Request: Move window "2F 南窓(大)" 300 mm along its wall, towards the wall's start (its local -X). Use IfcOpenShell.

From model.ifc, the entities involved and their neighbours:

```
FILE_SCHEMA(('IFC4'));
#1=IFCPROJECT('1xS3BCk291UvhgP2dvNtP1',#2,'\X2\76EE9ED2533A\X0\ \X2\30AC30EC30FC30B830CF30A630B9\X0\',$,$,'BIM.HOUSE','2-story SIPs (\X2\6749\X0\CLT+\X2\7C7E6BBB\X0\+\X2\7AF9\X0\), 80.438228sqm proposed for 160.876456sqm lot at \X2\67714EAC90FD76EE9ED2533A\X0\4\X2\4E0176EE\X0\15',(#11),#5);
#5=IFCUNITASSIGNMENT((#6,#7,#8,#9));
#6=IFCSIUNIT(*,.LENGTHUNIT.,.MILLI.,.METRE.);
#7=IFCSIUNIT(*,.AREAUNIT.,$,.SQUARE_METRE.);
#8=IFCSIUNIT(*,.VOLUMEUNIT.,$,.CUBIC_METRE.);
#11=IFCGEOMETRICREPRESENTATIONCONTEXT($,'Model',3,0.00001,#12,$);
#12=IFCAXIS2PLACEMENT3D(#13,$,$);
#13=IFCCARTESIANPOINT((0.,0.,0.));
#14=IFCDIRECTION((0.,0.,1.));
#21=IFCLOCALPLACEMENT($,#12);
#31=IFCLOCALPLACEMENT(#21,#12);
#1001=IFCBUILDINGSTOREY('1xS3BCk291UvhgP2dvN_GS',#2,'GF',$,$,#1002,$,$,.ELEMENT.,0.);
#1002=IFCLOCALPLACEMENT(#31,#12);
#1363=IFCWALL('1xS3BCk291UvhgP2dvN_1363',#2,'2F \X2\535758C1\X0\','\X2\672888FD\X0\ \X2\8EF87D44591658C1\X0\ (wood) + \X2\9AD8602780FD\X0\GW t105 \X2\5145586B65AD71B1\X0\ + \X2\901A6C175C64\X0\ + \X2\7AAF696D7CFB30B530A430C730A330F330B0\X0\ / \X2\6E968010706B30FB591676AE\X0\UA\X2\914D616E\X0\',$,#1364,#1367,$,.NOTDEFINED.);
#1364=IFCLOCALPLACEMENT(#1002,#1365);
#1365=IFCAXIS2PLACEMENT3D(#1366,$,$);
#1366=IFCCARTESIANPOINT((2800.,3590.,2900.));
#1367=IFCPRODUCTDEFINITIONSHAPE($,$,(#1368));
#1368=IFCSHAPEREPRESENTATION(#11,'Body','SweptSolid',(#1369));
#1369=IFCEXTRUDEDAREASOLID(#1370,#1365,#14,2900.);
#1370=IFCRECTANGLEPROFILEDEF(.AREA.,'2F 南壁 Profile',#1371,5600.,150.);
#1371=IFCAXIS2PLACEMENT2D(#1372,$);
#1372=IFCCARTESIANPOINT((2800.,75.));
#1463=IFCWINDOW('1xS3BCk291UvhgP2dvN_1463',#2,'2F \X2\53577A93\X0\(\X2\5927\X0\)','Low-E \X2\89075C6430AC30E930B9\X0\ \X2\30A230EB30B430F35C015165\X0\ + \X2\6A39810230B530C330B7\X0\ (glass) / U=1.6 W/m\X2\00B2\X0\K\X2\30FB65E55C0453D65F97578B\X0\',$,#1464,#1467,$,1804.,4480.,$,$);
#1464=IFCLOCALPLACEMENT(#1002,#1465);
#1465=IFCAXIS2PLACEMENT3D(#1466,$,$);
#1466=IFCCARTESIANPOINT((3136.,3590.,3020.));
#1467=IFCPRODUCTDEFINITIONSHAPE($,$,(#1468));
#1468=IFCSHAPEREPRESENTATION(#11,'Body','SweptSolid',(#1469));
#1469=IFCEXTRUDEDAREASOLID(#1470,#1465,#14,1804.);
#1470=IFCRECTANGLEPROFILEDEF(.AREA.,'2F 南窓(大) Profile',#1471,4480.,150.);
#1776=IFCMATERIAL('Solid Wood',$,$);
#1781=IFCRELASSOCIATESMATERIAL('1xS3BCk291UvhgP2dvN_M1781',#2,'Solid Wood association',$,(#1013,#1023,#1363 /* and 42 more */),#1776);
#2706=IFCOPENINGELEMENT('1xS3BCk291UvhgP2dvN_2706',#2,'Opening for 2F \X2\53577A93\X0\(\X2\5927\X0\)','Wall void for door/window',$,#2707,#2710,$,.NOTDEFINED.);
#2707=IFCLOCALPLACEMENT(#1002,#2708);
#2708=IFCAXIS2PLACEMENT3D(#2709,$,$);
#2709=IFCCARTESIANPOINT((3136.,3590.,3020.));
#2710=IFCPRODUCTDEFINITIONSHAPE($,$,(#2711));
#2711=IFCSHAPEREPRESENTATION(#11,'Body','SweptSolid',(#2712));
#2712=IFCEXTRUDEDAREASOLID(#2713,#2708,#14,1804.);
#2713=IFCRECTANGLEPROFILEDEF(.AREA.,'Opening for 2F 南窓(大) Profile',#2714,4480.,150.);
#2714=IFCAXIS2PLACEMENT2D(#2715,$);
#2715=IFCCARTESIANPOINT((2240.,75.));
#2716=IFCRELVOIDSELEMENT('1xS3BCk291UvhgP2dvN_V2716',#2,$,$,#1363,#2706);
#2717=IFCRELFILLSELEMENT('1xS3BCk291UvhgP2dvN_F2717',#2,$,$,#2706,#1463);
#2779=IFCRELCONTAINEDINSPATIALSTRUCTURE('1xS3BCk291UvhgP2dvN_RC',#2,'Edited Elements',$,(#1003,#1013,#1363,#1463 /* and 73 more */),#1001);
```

```python
import ifcopenshell
import ifcopenshell.api.geometry
import ifcopenshell.util.placement

model = ifcopenshell.open("model.ifc")

window = model.by_id(1463)
opening = window.FillsVoids[0].RelatingOpeningElement
wall = opening.VoidsElements[0].RelatingBuildingElement

wall_matrix = ifcopenshell.util.placement.get_local_placement(wall.ObjectPlacement)
shift = wall_matrix[:3, 0] * -300.0
before = ifcopenshell.util.placement.get_local_placement(window.ObjectPlacement)[:3, 3].copy()

# The window is not placed relative to its opening, so move both.
for product in (opening, window):
    matrix = ifcopenshell.util.placement.get_local_placement(product.ObjectPlacement)
    matrix[:3, 3] += shift
    ifcopenshell.api.geometry.edit_object_placement(model, product=product, matrix=matrix, is_si=False)

after = ifcopenshell.util.placement.get_local_placement(window.ObjectPlacement)[:3, 3]
print("window moved by", (after - before).round(3) + 0.0)

model.write("model_rev.ifc")
```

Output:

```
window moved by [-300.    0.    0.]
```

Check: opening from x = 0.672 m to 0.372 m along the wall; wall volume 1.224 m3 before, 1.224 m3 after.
